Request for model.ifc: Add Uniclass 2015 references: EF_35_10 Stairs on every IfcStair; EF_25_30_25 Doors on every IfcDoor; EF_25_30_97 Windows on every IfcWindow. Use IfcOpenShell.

First a look at what the model holds.

```python
import ifcopenshell

model = ifcopenshell.open("model.ifc")
print(model.schema)
print("classifications:", [c.Name for c in model.by_type("IfcClassification")])
for ifc_class in ("IfcDoor", "IfcRoof", "IfcStair", "IfcWall", "IfcWindow"):
    print(ifc_class, len(model.by_type(ifc_class)))
```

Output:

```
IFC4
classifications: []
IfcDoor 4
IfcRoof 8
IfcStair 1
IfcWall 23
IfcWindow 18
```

```python
import ifcopenshell
import ifcopenshell.api.classification

model = ifcopenshell.open("model.ifc")

system = ifcopenshell.api.classification.add_classification(model, classification="Uniclass 2015")

codes = {
    "IfcStair": ("EF_35_10", "Stairs"),
    "IfcDoor": ("EF_25_30_25", "Doors"),
    "IfcWindow": ("EF_25_30_97", "Windows"),
}
for ifc_class, (code, name) in codes.items():
    products = model.by_type(ifc_class)
    ifcopenshell.api.classification.add_reference(
        model, products=products, classification=system, identification=code, name=name
    )
    print(code, len(products))

model.write("model_rev.ifc")
```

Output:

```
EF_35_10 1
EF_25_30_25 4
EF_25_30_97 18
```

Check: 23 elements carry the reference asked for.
